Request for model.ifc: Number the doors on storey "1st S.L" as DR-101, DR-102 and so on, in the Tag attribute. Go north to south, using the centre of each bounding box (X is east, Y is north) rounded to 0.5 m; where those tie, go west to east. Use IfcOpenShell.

First a look at what the model holds.

```python
import ifcopenshell
import ifcopenshell.util.element
import ifcopenshell.util.placement

model = ifcopenshell.open("model.ifc")
print(model.schema)
storey = next(s for s in model.by_type("IfcBuildingStorey") if s.Name == "1st S.L")
doors = [e for e in ifcopenshell.util.element.get_decomposition(storey) if e.is_a("IfcDoor")]
for e in sorted(doors, key=lambda e: e.id()):
    origin = ifcopenshell.util.placement.get_local_placement(e.ObjectPlacement)[:3, 3]
    print(e.id(), e.Tag, e.Name, origin.round(2) + 0.0, sep=" | ")
```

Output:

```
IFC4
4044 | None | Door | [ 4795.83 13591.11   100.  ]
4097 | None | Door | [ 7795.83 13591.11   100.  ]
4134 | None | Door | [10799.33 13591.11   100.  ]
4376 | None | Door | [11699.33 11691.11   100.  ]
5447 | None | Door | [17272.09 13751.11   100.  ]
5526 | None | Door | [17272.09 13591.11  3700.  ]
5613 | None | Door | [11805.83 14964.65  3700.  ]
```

```python
import ifcopenshell
import ifcopenshell.geom
import ifcopenshell.util.element
import ifcopenshell.util.shape

model = ifcopenshell.open("model.ifc")
settings = ifcopenshell.geom.settings()
settings.set("use-world-coords", True)


def centre(element):
    shape = ifcopenshell.geom.create_shape(settings, element)
    return ifcopenshell.util.shape.get_bbox_centroid(shape.geometry)


storey = next(s for s in model.by_type("IfcBuildingStorey") if s.Name == "1st S.L")
doors = [e for e in ifcopenshell.util.element.get_decomposition(storey) if e.is_a("IfcDoor")]

# Insertion points can sit at a corner or the storey origin, so sort by the geometry (in metres).
centres = {e: centre(e) for e in doors}
doors.sort(key=lambda e: (-round(centres[e][1] / 0.5), centres[e][0]))

for i, e in enumerate(doors, start=1):
    number = f"DR-1{i:02d}"
    e.Tag = number
    print(e.id(), number)

model.write("model_updated.ifc")
```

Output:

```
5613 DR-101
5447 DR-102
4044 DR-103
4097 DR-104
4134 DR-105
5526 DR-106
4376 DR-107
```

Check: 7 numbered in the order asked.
